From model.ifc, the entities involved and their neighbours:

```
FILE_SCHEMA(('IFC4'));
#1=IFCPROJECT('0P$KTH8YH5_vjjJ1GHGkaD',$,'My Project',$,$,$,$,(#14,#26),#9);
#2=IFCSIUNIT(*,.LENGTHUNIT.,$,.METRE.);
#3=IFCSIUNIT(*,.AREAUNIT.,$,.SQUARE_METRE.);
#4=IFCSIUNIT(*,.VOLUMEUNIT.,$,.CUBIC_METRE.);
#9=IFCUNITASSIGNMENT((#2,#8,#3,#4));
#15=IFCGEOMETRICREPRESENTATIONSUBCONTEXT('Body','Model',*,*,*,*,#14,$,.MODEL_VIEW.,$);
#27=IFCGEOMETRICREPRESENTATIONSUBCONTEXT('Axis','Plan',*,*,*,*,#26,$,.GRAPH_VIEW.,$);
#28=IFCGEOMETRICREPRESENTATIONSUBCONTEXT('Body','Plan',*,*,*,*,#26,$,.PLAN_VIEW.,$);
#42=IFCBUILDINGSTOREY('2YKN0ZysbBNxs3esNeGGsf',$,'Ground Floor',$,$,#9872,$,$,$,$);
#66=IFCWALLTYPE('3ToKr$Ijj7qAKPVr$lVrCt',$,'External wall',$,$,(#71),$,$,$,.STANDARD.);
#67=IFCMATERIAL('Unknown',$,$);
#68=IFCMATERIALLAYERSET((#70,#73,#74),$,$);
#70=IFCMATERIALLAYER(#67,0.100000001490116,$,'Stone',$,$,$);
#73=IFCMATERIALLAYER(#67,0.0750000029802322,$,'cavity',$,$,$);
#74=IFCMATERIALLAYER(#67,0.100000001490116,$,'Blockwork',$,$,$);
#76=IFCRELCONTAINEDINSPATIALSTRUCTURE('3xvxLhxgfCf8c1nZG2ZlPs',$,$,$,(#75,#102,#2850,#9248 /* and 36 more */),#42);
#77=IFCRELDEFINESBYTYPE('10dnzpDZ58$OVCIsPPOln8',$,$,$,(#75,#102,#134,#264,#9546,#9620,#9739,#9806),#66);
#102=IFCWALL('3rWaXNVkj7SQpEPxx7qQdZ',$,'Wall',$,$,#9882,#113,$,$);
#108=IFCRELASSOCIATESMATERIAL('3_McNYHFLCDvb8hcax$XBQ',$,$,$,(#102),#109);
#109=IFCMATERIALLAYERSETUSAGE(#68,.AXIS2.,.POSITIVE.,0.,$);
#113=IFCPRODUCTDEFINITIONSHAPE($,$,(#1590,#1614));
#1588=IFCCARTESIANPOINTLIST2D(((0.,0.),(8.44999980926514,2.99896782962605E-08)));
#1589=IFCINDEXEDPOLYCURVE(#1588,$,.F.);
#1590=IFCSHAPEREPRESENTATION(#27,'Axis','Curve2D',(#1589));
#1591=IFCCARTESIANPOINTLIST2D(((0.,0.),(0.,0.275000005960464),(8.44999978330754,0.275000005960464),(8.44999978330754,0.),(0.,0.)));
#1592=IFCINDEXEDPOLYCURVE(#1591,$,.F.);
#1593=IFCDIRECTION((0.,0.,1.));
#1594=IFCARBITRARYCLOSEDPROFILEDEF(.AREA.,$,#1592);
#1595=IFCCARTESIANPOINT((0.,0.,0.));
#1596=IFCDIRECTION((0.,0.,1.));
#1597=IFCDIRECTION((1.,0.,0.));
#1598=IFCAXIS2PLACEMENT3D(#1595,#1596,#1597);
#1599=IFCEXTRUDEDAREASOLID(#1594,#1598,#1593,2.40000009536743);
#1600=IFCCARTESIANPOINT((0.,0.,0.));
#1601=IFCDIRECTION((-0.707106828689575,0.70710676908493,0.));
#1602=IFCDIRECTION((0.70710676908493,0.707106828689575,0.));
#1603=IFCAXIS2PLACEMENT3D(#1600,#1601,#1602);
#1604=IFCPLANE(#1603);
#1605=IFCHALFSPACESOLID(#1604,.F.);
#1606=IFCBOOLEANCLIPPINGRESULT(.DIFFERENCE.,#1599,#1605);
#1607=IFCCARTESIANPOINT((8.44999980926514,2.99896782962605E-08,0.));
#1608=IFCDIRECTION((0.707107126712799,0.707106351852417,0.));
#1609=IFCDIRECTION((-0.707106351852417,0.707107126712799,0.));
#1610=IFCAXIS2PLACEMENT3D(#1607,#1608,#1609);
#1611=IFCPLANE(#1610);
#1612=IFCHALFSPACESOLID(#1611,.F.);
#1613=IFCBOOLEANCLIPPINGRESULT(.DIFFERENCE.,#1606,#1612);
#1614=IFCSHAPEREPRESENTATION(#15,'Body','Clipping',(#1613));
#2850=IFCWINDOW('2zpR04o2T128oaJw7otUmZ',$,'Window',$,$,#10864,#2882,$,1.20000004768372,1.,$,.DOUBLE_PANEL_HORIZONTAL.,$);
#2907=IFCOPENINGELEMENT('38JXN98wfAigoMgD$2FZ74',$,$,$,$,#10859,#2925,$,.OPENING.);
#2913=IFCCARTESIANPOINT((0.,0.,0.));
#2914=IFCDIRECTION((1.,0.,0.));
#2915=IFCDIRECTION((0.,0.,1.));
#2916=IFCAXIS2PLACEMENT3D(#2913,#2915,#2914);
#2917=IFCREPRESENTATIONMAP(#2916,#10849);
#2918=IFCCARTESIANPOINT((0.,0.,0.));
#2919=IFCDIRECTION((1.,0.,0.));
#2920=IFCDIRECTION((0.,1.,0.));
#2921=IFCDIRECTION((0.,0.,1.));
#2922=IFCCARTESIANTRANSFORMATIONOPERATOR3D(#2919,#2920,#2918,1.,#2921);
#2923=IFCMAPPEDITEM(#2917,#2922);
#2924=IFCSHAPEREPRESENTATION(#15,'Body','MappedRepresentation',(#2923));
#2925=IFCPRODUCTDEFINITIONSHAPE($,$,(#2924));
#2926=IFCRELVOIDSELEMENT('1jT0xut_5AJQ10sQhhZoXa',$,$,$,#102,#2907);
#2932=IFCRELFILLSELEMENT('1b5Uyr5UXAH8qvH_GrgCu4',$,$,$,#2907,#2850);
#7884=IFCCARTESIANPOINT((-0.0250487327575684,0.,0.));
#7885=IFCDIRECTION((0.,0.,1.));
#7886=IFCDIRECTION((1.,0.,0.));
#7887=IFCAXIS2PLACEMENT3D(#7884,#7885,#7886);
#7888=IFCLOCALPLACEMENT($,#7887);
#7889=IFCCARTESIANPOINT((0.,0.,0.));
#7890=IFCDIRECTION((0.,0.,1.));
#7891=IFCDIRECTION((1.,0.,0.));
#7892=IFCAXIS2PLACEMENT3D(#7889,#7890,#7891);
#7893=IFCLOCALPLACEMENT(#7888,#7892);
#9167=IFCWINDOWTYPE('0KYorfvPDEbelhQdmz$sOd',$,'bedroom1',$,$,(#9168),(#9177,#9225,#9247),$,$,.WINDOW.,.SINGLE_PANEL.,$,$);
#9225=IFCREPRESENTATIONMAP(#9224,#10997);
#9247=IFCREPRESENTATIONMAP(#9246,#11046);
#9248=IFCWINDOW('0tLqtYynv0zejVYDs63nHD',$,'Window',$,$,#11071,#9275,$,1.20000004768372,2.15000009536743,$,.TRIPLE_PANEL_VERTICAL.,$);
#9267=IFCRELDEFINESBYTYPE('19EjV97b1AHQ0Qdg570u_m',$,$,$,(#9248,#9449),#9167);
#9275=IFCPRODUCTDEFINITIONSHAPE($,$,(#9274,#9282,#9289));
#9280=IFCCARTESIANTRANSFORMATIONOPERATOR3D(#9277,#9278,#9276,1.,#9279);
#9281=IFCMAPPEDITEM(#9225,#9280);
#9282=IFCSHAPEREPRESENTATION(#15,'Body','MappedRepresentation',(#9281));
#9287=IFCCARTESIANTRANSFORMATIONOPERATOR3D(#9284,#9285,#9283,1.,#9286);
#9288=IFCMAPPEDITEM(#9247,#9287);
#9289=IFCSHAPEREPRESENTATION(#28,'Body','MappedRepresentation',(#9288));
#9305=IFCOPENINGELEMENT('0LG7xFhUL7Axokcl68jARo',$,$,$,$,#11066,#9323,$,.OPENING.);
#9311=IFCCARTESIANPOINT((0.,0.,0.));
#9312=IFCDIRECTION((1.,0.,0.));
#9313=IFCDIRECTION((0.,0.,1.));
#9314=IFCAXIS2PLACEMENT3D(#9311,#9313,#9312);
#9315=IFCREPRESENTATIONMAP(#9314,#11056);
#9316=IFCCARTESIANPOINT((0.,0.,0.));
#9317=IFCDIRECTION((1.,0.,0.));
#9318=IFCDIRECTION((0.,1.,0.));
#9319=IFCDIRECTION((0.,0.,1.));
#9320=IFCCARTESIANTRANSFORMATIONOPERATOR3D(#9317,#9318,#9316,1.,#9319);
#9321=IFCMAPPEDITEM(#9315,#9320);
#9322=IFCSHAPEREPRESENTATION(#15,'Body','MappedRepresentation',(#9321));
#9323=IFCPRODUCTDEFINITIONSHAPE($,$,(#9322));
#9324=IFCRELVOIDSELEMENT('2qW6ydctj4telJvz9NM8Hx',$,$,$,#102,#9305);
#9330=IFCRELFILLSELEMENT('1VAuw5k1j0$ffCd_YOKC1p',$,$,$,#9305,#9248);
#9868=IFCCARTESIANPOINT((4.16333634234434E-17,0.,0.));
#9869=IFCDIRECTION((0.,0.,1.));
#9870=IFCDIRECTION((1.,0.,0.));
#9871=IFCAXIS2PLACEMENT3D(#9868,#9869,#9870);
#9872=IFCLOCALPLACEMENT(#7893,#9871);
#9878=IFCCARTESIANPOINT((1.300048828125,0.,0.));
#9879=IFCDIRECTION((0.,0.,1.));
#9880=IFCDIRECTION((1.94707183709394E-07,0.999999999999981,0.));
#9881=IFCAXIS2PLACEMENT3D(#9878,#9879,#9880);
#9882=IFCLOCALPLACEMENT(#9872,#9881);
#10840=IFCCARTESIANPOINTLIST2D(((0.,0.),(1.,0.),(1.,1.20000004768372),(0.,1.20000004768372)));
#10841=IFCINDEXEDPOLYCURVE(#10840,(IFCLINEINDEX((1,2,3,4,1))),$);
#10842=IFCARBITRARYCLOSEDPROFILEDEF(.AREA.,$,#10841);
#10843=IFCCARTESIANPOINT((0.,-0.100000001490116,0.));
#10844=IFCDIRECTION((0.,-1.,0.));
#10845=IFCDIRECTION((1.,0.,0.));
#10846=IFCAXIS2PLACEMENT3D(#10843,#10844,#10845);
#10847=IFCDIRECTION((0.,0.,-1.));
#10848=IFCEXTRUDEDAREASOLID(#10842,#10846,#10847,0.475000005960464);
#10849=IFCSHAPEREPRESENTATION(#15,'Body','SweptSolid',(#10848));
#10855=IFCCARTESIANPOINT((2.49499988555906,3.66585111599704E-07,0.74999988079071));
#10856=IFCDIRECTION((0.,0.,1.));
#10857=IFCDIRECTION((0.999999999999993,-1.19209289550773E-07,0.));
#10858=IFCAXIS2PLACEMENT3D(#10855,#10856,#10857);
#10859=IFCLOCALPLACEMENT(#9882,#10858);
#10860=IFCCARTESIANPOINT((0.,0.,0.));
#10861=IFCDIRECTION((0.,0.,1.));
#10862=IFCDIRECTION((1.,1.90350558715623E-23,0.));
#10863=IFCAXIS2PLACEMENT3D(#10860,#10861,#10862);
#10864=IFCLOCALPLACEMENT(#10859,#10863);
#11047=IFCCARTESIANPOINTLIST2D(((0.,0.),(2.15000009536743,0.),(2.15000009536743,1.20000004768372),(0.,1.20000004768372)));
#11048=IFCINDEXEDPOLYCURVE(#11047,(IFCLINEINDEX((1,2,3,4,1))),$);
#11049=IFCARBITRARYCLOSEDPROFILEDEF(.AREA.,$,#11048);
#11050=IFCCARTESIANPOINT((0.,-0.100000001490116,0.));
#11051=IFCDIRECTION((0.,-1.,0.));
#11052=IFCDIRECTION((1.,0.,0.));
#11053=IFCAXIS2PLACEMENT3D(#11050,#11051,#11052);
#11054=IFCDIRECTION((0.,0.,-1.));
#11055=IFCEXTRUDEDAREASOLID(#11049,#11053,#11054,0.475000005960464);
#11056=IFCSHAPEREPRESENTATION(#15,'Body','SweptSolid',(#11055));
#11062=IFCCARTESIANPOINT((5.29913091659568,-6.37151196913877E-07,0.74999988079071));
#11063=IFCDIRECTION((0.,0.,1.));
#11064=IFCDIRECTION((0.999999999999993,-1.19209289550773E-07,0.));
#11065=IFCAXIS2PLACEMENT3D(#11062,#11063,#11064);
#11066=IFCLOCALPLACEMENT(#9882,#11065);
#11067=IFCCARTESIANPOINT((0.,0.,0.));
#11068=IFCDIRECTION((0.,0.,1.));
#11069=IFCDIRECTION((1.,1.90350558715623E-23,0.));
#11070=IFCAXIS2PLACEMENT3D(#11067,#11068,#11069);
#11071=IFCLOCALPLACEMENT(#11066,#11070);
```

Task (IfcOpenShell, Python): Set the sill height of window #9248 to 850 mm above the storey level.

```python
import numpy as np
import ifcopenshell
import ifcopenshell.api.geometry
import ifcopenshell.geom
import ifcopenshell.util.element
import ifcopenshell.util.placement
import ifcopenshell.util.shape
import ifcopenshell.util.unit

model = ifcopenshell.open("model.ifc")
unit_scale = ifcopenshell.util.unit.calculate_unit_scale(model)

window = model.by_guid("0tLqtYynv0zejVYDs63nHD")
opening = window.FillsVoids[0].RelatingOpeningElement
storey = ifcopenshell.util.element.get_container(window, ifc_class="IfcBuildingStorey")
level = ifcopenshell.util.placement.get_local_placement(storey.ObjectPlacement)[2, 3]

# The opening's origin need not be at the sill, so measure its lowest point.
shape = ifcopenshell.geom.create_shape(ifcopenshell.geom.settings(), opening)
bottom = ifcopenshell.util.shape.get_shape_bottom_elevation(shape, shape.geometry) / unit_scale
dz = level + 0.85 - bottom

shift = np.array([0.0, 0.0, dz])
# The window is placed relative to its opening, so it follows when the opening moves.
matrix = ifcopenshell.util.placement.get_local_placement(opening.ObjectPlacement)
matrix[:3, 3] += shift
ifcopenshell.api.geometry.edit_object_placement(
    model, product=opening, matrix=matrix, is_si=False, should_transform_children=True
)

print(f"moved by {dz * unit_scale:+.3f} m")

model.write("model_updated.ifc")
```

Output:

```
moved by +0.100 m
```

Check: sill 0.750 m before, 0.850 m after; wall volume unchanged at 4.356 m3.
